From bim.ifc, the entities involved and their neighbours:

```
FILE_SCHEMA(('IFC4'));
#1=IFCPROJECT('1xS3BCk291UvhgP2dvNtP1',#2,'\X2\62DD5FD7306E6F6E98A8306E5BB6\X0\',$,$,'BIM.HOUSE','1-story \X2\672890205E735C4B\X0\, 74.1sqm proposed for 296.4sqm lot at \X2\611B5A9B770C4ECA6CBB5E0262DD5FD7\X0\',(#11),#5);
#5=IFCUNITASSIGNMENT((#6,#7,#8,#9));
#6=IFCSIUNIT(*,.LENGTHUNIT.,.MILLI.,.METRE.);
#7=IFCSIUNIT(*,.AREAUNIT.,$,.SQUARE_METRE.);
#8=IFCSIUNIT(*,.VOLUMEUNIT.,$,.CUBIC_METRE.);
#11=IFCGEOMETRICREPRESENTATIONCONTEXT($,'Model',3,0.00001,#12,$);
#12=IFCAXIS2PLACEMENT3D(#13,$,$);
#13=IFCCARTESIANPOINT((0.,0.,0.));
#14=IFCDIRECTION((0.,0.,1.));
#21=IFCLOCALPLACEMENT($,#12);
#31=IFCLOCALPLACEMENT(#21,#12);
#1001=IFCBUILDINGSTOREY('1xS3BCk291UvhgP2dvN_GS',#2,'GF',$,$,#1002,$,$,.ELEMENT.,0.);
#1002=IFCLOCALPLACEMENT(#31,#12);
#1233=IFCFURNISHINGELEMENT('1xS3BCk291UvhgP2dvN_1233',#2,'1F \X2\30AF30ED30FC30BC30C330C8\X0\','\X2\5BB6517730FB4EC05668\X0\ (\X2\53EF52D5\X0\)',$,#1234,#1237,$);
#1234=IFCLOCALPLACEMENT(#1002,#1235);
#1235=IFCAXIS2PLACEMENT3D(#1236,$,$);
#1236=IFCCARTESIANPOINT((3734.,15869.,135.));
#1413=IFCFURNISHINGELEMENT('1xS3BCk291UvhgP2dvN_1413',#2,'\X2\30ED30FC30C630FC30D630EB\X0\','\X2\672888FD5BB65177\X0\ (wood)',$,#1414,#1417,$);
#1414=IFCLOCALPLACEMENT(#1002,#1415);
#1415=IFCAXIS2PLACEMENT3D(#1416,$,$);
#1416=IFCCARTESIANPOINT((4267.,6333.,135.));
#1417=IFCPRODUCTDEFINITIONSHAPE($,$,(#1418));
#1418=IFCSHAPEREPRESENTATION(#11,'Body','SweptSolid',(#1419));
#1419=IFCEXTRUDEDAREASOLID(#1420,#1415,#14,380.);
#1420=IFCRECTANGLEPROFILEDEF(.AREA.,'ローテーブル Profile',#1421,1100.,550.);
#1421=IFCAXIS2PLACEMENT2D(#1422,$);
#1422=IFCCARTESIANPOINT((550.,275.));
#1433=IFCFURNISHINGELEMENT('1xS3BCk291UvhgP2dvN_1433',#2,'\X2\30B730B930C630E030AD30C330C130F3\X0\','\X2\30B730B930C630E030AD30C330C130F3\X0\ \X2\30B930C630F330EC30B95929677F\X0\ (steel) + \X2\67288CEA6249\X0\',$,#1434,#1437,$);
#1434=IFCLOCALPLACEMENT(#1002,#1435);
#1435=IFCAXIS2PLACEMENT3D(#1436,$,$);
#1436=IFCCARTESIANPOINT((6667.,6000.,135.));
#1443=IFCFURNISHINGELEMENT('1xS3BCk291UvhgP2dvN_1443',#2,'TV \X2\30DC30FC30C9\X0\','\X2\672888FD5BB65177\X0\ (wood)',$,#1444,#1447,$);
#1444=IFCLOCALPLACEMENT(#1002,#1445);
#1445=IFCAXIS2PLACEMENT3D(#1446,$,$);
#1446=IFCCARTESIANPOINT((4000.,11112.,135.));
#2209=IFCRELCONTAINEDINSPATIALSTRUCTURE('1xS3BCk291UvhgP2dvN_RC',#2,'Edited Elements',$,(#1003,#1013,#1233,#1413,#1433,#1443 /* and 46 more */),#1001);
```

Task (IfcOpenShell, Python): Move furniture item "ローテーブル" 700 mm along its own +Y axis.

```python
import ifcopenshell
import ifcopenshell.api.geometry
import ifcopenshell.util.placement
import ifcopenshell.util.unit

model = ifcopenshell.open("bim.ifc")
unit_scale = ifcopenshell.util.unit.calculate_unit_scale(model)

item = model.by_guid("1xS3BCk291UvhgP2dvN_1413")
matrix = ifcopenshell.util.placement.get_local_placement(item.ObjectPlacement)
matrix[:3, 3] += matrix[:3, 1] * 0.7 / unit_scale
ifcopenshell.api.geometry.edit_object_placement(model, product=item, matrix=matrix, is_si=False)

print(ifcopenshell.util.placement.get_local_placement(item.ObjectPlacement).round(3) + 0.0)

model.write("bim_rev.ifc")
```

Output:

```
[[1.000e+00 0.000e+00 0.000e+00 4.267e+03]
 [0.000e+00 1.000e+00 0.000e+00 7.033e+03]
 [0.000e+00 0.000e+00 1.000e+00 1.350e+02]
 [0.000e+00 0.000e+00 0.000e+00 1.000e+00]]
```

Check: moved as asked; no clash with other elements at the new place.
